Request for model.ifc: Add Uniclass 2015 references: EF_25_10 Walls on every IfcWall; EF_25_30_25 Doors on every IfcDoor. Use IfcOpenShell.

First a look at what the model holds.

```python
import ifcopenshell

model = ifcopenshell.open("model.ifc")
print(model.schema)
print("classifications:", [c.Name for c in model.by_type("IfcClassification")])
for ifc_class in ("IfcDoor", "IfcRoof", "IfcStair", "IfcWall", "IfcWindow"):
    print(ifc_class, len(model.by_type(ifc_class)))
```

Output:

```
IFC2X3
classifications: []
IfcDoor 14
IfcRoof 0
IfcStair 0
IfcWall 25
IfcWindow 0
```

```python
import ifcopenshell
import ifcopenshell.api.classification

model = ifcopenshell.open("model.ifc")

# IFC2X3 requires Source and Edition and has no link from the project to the system.
system = model.create_entity("IfcClassification", Source="NBS", Edition="2015", Name="Uniclass 2015")

codes = {
    "IfcWall": ("EF_25_10", "Walls"),
    "IfcDoor": ("EF_25_30_25", "Doors"),
}
for ifc_class, (code, name) in codes.items():
    products = model.by_type(ifc_class)
    ifcopenshell.api.classification.add_reference(
        model, products=products, classification=system, identification=code, name=name
    )
    print(code, len(products))

model.write("model_rev.ifc")
```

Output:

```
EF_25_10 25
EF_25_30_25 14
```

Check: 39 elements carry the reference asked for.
